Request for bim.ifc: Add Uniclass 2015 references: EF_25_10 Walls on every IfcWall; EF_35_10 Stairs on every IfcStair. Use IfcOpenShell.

First a look at what the model holds.

```python
import ifcopenshell

model = ifcopenshell.open("bim.ifc")
print(model.schema)
print("classifications:", [c.Name for c in model.by_type("IfcClassification")])
for ifc_class in ("IfcDoor", "IfcRoof", "IfcStair", "IfcWall", "IfcWindow"):
    print(ifc_class, len(model.by_type(ifc_class)))
```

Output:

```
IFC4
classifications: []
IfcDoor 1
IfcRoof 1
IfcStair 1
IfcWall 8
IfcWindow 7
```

```python
import ifcopenshell
import ifcopenshell.api.classification

model = ifcopenshell.open("bim.ifc")

system = ifcopenshell.api.classification.add_classification(model, classification="Uniclass 2015")

codes = {
    "IfcWall": ("EF_25_10", "Walls"),
    "IfcStair": ("EF_35_10", "Stairs"),
}
for ifc_class, (code, name) in codes.items():
    products = model.by_type(ifc_class)
    ifcopenshell.api.classification.add_reference(
        model, products=products, classification=system, identification=code, name=name
    )
    print(code, len(products))

model.write("bim-out.ifc")
```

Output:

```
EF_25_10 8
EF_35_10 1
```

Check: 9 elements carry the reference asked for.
